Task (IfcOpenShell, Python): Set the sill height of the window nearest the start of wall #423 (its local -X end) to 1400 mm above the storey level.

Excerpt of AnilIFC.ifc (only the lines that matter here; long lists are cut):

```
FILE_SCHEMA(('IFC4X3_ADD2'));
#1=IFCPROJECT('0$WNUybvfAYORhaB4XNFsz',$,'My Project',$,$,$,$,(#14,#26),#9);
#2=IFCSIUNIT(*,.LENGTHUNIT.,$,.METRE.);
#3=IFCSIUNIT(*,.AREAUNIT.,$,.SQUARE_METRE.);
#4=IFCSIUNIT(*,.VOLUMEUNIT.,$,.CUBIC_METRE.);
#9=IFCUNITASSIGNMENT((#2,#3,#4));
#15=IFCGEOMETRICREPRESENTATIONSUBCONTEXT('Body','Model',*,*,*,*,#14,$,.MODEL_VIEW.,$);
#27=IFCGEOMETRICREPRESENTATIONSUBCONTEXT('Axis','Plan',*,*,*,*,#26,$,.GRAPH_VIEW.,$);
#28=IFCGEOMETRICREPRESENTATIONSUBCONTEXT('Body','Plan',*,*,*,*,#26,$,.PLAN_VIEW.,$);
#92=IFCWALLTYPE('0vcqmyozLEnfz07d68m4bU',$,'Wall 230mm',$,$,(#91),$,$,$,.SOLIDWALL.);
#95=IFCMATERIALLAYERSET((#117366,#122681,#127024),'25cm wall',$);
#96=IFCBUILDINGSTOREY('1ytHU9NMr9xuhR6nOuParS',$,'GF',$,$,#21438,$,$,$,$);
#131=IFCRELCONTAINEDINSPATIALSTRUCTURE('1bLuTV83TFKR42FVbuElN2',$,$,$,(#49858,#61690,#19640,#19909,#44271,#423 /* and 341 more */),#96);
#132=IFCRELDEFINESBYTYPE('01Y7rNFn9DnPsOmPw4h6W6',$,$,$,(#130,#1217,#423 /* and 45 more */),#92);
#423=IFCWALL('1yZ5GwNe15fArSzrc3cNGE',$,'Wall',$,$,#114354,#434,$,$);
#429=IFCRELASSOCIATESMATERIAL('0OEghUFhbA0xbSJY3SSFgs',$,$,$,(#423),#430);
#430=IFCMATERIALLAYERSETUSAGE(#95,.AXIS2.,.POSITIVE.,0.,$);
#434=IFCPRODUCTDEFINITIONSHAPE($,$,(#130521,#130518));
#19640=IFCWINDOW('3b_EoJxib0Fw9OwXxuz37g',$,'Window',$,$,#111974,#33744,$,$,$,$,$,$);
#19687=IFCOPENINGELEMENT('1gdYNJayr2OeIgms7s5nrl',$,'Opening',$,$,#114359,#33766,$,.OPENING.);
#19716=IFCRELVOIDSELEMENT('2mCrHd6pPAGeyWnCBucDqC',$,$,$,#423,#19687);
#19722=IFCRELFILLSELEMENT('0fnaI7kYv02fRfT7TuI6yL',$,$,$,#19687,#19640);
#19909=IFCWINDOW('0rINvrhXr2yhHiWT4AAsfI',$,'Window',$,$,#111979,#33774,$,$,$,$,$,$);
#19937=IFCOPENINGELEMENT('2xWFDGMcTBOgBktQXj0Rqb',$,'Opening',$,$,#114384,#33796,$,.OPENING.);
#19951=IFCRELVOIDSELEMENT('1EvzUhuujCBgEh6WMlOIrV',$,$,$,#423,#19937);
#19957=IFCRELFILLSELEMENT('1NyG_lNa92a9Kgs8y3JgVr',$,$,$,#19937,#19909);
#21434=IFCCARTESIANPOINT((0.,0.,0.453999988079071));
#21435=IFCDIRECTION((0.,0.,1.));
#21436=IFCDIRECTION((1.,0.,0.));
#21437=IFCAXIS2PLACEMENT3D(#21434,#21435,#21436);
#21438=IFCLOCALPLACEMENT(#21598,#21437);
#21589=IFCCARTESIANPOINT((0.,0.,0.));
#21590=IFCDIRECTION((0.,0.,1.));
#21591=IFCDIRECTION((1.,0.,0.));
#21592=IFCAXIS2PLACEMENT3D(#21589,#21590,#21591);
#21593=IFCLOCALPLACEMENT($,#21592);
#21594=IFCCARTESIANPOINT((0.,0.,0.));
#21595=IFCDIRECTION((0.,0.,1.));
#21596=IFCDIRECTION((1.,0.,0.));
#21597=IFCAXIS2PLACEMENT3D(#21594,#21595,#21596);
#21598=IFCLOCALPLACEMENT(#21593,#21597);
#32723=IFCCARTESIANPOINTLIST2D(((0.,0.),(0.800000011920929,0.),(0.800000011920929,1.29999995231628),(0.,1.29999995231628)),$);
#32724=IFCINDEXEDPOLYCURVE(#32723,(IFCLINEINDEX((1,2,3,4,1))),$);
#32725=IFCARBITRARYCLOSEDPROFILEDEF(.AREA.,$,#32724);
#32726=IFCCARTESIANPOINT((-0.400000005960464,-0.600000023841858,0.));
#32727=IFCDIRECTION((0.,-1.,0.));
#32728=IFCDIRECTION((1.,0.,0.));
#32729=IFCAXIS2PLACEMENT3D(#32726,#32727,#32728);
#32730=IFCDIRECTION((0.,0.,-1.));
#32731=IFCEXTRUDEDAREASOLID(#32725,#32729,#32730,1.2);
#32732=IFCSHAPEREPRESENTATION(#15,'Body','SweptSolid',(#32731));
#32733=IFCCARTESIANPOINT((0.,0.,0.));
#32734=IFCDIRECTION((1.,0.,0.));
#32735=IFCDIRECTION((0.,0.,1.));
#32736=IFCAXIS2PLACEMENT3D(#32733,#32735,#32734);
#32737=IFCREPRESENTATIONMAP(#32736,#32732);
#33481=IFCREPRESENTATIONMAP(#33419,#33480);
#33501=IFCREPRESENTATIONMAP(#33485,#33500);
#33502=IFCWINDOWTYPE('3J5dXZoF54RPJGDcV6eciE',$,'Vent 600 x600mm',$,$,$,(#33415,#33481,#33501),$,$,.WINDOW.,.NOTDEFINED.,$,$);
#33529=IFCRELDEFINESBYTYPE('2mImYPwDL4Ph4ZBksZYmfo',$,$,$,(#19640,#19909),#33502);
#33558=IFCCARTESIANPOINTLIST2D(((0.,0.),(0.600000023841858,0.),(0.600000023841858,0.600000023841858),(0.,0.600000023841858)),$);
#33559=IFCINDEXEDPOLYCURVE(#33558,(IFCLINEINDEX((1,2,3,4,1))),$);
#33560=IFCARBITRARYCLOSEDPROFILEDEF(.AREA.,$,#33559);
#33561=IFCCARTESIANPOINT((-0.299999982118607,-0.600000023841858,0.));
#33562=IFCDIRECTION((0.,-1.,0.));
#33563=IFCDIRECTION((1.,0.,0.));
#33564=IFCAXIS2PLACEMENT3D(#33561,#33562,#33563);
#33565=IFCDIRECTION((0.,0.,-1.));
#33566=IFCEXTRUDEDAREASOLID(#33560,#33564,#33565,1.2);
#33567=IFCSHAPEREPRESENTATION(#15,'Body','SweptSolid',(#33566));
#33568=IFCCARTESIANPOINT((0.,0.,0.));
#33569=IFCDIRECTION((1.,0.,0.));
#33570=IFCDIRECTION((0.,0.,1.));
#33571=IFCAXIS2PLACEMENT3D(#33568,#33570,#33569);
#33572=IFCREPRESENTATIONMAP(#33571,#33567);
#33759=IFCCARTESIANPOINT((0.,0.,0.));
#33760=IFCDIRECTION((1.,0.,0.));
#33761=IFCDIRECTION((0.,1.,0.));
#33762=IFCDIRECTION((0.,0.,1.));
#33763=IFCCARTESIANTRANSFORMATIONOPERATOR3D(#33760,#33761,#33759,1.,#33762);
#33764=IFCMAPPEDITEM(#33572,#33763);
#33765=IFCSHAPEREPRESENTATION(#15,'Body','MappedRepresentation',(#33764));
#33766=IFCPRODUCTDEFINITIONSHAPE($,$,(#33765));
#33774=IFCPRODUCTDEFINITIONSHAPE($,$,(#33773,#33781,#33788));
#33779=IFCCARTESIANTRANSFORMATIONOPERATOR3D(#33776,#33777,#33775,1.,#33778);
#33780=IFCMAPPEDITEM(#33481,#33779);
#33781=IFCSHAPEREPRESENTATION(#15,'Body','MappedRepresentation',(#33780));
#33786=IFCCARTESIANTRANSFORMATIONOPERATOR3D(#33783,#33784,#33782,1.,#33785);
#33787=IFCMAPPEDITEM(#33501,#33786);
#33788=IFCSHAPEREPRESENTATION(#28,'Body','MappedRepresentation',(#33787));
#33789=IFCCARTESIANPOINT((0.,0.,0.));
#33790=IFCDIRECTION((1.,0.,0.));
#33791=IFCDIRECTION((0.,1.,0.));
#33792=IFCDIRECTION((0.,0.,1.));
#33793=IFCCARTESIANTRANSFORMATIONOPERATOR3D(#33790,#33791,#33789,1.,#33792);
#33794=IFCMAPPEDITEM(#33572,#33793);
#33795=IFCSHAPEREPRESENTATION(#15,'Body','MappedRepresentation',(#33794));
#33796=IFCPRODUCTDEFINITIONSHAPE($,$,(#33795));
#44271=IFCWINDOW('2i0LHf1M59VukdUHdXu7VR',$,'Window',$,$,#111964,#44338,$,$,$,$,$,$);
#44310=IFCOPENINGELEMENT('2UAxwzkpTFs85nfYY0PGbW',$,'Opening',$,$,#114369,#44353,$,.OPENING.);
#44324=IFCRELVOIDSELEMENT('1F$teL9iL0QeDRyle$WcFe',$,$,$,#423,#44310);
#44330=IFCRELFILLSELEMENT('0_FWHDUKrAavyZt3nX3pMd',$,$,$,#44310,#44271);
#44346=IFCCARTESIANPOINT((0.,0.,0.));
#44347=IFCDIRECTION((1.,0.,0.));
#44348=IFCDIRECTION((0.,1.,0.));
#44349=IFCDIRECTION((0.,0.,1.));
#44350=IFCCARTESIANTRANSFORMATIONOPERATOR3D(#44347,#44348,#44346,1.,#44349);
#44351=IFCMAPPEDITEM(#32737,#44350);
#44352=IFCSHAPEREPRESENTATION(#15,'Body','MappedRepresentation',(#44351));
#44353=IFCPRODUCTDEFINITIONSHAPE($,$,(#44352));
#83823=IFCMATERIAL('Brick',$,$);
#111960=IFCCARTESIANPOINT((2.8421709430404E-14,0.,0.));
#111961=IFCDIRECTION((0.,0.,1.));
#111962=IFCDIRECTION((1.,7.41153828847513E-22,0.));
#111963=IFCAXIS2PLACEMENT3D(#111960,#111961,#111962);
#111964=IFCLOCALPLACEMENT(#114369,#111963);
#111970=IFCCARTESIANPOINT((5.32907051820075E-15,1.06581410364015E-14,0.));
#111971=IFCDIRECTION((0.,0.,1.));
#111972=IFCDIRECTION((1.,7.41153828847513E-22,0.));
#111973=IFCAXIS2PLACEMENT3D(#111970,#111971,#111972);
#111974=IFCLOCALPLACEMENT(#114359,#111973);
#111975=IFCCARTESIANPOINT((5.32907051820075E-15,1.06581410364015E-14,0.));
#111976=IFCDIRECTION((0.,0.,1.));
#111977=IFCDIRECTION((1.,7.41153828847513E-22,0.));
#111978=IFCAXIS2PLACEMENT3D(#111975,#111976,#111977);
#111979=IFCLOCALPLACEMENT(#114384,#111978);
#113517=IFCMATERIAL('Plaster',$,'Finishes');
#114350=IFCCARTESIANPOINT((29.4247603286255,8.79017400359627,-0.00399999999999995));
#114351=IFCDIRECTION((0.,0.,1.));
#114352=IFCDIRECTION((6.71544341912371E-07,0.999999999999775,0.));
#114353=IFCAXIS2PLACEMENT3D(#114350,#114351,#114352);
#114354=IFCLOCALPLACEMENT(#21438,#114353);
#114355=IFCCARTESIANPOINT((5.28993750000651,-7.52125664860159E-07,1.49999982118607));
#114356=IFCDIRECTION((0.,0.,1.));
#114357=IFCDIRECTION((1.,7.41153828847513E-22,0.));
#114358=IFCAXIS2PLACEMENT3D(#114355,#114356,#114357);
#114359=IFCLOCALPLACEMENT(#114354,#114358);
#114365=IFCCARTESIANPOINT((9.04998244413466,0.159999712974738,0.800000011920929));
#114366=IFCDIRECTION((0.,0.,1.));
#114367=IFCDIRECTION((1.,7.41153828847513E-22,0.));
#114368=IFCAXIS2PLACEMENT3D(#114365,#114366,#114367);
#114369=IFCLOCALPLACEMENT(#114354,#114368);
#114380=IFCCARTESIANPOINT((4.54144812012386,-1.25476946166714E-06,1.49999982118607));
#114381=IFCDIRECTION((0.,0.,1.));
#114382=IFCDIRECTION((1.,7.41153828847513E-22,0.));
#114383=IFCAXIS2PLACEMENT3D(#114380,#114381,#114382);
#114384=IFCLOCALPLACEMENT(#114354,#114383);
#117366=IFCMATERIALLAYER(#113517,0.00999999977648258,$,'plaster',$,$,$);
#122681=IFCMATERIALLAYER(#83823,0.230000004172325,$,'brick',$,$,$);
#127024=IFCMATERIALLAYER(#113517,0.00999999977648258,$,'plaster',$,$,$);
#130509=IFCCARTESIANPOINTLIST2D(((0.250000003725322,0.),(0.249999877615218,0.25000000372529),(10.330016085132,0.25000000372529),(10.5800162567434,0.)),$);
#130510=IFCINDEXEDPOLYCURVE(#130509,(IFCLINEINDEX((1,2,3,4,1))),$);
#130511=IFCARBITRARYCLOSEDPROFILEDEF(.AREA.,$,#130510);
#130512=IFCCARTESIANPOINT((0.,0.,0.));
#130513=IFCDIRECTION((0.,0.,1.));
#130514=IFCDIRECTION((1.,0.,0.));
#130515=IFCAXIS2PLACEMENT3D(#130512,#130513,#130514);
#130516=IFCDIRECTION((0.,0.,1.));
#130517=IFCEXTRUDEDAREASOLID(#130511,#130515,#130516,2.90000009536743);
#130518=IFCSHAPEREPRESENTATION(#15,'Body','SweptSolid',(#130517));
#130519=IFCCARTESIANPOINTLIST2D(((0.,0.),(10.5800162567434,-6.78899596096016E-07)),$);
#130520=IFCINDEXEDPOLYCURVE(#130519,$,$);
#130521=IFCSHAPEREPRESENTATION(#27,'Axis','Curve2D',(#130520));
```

```python
import numpy as np
import ifcopenshell
import ifcopenshell.api.geometry
import ifcopenshell.geom
import ifcopenshell.util.element
import ifcopenshell.util.placement
import ifcopenshell.util.shape
import ifcopenshell.util.unit

model = ifcopenshell.open("AnilIFC.ifc")
unit_scale = ifcopenshell.util.unit.calculate_unit_scale(model)

window = model.by_guid("0rINvrhXr2yhHiWT4AAsfI")
opening = window.FillsVoids[0].RelatingOpeningElement
storey = ifcopenshell.util.element.get_container(window, ifc_class="IfcBuildingStorey")
level = ifcopenshell.util.placement.get_local_placement(storey.ObjectPlacement)[2, 3]

# The opening's origin need not be at the sill, so measure its lowest point.
shape = ifcopenshell.geom.create_shape(ifcopenshell.geom.settings(), opening)
bottom = ifcopenshell.util.shape.get_shape_bottom_elevation(shape, shape.geometry) / unit_scale
dz = level + 1.4 / unit_scale - bottom

shift = np.array([0.0, 0.0, dz])
# The window is placed relative to its opening, so it follows when the opening moves.
matrix = ifcopenshell.util.placement.get_local_placement(opening.ObjectPlacement)
matrix[:3, 3] += shift
ifcopenshell.api.geometry.edit_object_placement(
    model, product=opening, matrix=matrix, is_si=False, should_transform_children=True
)

print(f"moved by {dz * unit_scale:+.3f} m")

model.write("AnilIFC_rev.ifc")
```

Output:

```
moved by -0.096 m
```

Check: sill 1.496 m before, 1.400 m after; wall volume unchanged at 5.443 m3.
